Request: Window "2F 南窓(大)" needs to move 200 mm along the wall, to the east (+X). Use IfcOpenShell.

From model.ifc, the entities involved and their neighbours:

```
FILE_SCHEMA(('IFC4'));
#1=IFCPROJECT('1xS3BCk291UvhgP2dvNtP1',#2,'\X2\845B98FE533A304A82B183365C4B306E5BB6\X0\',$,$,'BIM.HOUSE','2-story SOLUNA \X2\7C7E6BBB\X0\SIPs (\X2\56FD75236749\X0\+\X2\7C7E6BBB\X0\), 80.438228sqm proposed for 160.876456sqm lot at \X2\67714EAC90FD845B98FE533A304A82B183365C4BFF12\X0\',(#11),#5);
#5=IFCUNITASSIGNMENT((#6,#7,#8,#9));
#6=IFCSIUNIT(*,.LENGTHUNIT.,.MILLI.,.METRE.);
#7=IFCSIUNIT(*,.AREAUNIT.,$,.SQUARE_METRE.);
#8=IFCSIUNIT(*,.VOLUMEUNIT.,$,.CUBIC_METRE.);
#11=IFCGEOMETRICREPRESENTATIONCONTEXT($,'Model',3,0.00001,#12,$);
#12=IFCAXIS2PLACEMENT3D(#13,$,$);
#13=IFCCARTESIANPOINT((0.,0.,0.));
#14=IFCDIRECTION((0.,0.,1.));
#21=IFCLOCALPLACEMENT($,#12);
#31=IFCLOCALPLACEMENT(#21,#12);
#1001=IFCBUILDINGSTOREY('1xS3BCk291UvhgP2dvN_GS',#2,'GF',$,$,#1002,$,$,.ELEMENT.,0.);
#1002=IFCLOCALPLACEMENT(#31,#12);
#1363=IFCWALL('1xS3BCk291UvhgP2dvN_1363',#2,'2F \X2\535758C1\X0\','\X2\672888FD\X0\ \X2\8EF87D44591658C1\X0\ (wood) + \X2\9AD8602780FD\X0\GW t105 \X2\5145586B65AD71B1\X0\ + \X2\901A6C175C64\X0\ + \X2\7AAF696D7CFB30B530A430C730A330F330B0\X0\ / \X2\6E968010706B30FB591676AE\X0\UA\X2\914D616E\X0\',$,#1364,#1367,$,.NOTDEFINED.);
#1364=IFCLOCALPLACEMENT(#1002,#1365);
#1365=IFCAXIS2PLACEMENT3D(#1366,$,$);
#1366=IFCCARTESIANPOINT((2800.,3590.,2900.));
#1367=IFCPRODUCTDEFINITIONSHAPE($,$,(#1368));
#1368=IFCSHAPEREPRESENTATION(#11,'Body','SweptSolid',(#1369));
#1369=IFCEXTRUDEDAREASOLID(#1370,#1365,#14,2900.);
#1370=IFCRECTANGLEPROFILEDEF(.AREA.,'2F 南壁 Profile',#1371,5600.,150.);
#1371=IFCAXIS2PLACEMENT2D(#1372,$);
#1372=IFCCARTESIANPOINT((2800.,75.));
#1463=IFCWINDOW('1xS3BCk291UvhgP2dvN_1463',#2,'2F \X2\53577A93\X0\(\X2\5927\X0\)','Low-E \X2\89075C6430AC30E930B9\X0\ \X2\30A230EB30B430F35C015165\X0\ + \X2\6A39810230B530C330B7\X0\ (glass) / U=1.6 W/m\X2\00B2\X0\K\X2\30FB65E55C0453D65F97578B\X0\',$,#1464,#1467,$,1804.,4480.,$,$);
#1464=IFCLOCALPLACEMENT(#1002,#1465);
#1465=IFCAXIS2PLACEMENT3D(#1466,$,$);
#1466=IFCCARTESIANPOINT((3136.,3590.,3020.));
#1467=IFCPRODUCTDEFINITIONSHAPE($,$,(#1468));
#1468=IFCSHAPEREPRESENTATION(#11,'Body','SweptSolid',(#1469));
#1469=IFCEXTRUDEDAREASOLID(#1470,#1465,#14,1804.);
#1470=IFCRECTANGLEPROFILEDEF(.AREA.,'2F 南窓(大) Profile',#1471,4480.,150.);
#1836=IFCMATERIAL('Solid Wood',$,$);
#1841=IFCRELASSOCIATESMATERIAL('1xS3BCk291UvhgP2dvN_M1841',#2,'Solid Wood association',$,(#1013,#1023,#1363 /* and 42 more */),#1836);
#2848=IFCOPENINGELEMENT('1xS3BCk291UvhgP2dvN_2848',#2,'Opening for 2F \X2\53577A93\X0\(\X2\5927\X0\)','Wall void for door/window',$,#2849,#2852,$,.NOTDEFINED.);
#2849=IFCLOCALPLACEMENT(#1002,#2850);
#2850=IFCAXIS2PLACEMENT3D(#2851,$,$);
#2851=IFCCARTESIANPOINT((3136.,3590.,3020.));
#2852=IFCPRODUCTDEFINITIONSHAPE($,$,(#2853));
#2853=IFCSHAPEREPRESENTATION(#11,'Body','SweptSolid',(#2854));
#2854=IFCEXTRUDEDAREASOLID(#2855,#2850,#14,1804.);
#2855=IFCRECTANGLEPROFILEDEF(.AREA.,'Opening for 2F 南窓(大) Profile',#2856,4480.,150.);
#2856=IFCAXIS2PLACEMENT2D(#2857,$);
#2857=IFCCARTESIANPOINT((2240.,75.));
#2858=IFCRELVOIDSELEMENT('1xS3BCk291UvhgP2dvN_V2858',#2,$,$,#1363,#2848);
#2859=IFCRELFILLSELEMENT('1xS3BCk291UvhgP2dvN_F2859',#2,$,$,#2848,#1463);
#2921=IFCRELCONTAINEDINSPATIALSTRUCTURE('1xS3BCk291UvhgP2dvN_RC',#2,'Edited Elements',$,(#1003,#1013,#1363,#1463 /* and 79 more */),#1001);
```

```python
import ifcopenshell
import ifcopenshell.api.geometry
import ifcopenshell.util.placement
import ifcopenshell.util.unit

model = ifcopenshell.open("model.ifc")
unit_scale = ifcopenshell.util.unit.calculate_unit_scale(model)

window = model.by_guid("1xS3BCk291UvhgP2dvN_1463")
opening = window.FillsVoids[0].RelatingOpeningElement
wall = opening.VoidsElements[0].RelatingBuildingElement

wall_matrix = ifcopenshell.util.placement.get_local_placement(wall.ObjectPlacement)
shift = wall_matrix[:3, 0] * 0.2 / unit_scale
before = ifcopenshell.util.placement.get_local_placement(window.ObjectPlacement)[:3, 3].copy()

# The window is not placed relative to its opening, so move both.
for product in (opening, window):
    matrix = ifcopenshell.util.placement.get_local_placement(product.ObjectPlacement)
    matrix[:3, 3] += shift
    ifcopenshell.api.geometry.edit_object_placement(model, product=product, matrix=matrix, is_si=False)

after = ifcopenshell.util.placement.get_local_placement(window.ObjectPlacement)[:3, 3]
print("window moved by", (after - before).round(3) + 0.0)

model.write("model-out.ifc")
```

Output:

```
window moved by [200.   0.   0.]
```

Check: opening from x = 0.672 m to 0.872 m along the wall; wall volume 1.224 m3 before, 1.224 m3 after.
